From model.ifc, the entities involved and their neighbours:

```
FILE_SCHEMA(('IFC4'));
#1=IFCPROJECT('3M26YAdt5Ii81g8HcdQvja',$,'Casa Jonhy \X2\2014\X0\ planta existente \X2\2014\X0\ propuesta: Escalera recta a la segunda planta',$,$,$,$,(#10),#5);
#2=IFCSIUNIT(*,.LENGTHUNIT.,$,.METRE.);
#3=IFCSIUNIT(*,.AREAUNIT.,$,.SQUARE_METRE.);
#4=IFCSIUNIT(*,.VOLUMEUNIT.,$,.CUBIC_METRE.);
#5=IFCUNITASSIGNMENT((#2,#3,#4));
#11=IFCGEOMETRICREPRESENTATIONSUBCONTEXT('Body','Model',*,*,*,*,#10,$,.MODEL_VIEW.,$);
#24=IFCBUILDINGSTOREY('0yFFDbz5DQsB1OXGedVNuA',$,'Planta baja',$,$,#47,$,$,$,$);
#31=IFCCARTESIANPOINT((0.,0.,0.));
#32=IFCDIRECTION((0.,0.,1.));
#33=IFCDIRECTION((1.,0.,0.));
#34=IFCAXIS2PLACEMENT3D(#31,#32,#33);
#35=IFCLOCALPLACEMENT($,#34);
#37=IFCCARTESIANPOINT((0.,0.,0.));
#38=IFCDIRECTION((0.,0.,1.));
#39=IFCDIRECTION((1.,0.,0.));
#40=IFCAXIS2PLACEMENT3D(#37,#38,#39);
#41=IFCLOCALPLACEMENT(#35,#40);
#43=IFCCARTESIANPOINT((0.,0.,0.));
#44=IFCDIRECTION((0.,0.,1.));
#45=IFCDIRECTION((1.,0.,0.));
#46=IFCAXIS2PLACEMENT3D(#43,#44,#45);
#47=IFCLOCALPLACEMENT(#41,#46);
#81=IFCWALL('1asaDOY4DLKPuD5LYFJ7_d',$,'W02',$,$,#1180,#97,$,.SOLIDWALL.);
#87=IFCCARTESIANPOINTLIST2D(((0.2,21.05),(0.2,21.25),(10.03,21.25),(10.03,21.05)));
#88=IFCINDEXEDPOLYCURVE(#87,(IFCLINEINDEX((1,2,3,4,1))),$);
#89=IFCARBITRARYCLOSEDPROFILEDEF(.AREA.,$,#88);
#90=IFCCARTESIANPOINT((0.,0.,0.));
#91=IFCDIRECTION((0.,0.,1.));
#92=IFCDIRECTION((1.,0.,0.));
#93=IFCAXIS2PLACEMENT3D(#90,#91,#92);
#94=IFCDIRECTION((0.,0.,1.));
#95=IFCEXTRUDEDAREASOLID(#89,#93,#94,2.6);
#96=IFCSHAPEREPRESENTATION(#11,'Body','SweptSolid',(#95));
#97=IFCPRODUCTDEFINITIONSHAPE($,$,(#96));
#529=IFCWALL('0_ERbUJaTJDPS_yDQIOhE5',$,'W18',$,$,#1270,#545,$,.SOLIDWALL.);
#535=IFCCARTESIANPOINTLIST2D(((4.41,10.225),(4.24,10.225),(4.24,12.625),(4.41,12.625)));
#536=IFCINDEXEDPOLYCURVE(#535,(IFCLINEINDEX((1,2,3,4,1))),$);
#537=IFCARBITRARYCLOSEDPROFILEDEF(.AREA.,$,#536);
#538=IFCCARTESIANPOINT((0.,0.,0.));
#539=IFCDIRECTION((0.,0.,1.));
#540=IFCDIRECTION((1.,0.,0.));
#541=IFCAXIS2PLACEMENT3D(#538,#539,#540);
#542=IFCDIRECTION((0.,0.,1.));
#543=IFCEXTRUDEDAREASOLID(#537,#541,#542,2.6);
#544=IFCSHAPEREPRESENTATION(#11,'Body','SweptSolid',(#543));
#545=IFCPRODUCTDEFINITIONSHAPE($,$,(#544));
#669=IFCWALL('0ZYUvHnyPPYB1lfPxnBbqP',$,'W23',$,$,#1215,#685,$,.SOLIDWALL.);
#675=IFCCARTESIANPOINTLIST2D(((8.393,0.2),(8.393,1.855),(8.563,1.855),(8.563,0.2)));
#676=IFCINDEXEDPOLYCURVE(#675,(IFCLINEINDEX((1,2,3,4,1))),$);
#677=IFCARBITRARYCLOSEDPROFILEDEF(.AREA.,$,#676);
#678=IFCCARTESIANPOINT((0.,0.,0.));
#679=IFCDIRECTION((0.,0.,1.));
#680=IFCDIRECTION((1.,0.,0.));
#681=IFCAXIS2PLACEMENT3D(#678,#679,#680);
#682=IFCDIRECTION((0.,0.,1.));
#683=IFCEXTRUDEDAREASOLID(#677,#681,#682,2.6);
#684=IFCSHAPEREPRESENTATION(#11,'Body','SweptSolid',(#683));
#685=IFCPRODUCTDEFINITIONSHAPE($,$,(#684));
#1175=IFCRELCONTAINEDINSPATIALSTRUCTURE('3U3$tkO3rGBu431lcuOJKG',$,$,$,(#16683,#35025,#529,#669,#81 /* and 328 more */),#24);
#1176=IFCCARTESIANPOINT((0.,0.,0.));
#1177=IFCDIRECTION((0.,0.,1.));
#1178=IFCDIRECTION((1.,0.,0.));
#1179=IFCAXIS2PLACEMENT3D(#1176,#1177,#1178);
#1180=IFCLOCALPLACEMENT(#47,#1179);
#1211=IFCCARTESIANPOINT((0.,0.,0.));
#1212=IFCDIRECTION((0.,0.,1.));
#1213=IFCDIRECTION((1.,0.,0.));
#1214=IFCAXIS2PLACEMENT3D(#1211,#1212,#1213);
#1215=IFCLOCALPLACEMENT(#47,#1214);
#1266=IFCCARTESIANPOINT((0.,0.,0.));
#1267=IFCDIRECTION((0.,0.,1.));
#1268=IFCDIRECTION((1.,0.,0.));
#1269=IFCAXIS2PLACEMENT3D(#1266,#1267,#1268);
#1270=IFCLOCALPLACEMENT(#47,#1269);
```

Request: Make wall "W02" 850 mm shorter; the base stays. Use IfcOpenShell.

```python
import ifcopenshell
import ifcopenshell.geom
import ifcopenshell.util.representation
import ifcopenshell.util.shape

model = ifcopenshell.open("model.ifc")
settings = ifcopenshell.geom.settings()


def volume(element):
    """Net volume in cubic metres, openings subtracted."""
    shape = ifcopenshell.geom.create_shape(settings, element)
    return ifcopenshell.util.shape.get_volume(shape.geometry)


wall = model.by_id(81)
before = volume(wall)

body = ifcopenshell.util.representation.get_representation(wall, "Model", "Body")
solid = body.Items[0]
old_height = solid.Depth
solid.Depth -= 0.85
after = volume(wall)

print(f"height {old_height:g} -> {solid.Depth:g}, volume {before:.3f} -> {after:.3f} m3")

model.write("model_edited.ifc")
```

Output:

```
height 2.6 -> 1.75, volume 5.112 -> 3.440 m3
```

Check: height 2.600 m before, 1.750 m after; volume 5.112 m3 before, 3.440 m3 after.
